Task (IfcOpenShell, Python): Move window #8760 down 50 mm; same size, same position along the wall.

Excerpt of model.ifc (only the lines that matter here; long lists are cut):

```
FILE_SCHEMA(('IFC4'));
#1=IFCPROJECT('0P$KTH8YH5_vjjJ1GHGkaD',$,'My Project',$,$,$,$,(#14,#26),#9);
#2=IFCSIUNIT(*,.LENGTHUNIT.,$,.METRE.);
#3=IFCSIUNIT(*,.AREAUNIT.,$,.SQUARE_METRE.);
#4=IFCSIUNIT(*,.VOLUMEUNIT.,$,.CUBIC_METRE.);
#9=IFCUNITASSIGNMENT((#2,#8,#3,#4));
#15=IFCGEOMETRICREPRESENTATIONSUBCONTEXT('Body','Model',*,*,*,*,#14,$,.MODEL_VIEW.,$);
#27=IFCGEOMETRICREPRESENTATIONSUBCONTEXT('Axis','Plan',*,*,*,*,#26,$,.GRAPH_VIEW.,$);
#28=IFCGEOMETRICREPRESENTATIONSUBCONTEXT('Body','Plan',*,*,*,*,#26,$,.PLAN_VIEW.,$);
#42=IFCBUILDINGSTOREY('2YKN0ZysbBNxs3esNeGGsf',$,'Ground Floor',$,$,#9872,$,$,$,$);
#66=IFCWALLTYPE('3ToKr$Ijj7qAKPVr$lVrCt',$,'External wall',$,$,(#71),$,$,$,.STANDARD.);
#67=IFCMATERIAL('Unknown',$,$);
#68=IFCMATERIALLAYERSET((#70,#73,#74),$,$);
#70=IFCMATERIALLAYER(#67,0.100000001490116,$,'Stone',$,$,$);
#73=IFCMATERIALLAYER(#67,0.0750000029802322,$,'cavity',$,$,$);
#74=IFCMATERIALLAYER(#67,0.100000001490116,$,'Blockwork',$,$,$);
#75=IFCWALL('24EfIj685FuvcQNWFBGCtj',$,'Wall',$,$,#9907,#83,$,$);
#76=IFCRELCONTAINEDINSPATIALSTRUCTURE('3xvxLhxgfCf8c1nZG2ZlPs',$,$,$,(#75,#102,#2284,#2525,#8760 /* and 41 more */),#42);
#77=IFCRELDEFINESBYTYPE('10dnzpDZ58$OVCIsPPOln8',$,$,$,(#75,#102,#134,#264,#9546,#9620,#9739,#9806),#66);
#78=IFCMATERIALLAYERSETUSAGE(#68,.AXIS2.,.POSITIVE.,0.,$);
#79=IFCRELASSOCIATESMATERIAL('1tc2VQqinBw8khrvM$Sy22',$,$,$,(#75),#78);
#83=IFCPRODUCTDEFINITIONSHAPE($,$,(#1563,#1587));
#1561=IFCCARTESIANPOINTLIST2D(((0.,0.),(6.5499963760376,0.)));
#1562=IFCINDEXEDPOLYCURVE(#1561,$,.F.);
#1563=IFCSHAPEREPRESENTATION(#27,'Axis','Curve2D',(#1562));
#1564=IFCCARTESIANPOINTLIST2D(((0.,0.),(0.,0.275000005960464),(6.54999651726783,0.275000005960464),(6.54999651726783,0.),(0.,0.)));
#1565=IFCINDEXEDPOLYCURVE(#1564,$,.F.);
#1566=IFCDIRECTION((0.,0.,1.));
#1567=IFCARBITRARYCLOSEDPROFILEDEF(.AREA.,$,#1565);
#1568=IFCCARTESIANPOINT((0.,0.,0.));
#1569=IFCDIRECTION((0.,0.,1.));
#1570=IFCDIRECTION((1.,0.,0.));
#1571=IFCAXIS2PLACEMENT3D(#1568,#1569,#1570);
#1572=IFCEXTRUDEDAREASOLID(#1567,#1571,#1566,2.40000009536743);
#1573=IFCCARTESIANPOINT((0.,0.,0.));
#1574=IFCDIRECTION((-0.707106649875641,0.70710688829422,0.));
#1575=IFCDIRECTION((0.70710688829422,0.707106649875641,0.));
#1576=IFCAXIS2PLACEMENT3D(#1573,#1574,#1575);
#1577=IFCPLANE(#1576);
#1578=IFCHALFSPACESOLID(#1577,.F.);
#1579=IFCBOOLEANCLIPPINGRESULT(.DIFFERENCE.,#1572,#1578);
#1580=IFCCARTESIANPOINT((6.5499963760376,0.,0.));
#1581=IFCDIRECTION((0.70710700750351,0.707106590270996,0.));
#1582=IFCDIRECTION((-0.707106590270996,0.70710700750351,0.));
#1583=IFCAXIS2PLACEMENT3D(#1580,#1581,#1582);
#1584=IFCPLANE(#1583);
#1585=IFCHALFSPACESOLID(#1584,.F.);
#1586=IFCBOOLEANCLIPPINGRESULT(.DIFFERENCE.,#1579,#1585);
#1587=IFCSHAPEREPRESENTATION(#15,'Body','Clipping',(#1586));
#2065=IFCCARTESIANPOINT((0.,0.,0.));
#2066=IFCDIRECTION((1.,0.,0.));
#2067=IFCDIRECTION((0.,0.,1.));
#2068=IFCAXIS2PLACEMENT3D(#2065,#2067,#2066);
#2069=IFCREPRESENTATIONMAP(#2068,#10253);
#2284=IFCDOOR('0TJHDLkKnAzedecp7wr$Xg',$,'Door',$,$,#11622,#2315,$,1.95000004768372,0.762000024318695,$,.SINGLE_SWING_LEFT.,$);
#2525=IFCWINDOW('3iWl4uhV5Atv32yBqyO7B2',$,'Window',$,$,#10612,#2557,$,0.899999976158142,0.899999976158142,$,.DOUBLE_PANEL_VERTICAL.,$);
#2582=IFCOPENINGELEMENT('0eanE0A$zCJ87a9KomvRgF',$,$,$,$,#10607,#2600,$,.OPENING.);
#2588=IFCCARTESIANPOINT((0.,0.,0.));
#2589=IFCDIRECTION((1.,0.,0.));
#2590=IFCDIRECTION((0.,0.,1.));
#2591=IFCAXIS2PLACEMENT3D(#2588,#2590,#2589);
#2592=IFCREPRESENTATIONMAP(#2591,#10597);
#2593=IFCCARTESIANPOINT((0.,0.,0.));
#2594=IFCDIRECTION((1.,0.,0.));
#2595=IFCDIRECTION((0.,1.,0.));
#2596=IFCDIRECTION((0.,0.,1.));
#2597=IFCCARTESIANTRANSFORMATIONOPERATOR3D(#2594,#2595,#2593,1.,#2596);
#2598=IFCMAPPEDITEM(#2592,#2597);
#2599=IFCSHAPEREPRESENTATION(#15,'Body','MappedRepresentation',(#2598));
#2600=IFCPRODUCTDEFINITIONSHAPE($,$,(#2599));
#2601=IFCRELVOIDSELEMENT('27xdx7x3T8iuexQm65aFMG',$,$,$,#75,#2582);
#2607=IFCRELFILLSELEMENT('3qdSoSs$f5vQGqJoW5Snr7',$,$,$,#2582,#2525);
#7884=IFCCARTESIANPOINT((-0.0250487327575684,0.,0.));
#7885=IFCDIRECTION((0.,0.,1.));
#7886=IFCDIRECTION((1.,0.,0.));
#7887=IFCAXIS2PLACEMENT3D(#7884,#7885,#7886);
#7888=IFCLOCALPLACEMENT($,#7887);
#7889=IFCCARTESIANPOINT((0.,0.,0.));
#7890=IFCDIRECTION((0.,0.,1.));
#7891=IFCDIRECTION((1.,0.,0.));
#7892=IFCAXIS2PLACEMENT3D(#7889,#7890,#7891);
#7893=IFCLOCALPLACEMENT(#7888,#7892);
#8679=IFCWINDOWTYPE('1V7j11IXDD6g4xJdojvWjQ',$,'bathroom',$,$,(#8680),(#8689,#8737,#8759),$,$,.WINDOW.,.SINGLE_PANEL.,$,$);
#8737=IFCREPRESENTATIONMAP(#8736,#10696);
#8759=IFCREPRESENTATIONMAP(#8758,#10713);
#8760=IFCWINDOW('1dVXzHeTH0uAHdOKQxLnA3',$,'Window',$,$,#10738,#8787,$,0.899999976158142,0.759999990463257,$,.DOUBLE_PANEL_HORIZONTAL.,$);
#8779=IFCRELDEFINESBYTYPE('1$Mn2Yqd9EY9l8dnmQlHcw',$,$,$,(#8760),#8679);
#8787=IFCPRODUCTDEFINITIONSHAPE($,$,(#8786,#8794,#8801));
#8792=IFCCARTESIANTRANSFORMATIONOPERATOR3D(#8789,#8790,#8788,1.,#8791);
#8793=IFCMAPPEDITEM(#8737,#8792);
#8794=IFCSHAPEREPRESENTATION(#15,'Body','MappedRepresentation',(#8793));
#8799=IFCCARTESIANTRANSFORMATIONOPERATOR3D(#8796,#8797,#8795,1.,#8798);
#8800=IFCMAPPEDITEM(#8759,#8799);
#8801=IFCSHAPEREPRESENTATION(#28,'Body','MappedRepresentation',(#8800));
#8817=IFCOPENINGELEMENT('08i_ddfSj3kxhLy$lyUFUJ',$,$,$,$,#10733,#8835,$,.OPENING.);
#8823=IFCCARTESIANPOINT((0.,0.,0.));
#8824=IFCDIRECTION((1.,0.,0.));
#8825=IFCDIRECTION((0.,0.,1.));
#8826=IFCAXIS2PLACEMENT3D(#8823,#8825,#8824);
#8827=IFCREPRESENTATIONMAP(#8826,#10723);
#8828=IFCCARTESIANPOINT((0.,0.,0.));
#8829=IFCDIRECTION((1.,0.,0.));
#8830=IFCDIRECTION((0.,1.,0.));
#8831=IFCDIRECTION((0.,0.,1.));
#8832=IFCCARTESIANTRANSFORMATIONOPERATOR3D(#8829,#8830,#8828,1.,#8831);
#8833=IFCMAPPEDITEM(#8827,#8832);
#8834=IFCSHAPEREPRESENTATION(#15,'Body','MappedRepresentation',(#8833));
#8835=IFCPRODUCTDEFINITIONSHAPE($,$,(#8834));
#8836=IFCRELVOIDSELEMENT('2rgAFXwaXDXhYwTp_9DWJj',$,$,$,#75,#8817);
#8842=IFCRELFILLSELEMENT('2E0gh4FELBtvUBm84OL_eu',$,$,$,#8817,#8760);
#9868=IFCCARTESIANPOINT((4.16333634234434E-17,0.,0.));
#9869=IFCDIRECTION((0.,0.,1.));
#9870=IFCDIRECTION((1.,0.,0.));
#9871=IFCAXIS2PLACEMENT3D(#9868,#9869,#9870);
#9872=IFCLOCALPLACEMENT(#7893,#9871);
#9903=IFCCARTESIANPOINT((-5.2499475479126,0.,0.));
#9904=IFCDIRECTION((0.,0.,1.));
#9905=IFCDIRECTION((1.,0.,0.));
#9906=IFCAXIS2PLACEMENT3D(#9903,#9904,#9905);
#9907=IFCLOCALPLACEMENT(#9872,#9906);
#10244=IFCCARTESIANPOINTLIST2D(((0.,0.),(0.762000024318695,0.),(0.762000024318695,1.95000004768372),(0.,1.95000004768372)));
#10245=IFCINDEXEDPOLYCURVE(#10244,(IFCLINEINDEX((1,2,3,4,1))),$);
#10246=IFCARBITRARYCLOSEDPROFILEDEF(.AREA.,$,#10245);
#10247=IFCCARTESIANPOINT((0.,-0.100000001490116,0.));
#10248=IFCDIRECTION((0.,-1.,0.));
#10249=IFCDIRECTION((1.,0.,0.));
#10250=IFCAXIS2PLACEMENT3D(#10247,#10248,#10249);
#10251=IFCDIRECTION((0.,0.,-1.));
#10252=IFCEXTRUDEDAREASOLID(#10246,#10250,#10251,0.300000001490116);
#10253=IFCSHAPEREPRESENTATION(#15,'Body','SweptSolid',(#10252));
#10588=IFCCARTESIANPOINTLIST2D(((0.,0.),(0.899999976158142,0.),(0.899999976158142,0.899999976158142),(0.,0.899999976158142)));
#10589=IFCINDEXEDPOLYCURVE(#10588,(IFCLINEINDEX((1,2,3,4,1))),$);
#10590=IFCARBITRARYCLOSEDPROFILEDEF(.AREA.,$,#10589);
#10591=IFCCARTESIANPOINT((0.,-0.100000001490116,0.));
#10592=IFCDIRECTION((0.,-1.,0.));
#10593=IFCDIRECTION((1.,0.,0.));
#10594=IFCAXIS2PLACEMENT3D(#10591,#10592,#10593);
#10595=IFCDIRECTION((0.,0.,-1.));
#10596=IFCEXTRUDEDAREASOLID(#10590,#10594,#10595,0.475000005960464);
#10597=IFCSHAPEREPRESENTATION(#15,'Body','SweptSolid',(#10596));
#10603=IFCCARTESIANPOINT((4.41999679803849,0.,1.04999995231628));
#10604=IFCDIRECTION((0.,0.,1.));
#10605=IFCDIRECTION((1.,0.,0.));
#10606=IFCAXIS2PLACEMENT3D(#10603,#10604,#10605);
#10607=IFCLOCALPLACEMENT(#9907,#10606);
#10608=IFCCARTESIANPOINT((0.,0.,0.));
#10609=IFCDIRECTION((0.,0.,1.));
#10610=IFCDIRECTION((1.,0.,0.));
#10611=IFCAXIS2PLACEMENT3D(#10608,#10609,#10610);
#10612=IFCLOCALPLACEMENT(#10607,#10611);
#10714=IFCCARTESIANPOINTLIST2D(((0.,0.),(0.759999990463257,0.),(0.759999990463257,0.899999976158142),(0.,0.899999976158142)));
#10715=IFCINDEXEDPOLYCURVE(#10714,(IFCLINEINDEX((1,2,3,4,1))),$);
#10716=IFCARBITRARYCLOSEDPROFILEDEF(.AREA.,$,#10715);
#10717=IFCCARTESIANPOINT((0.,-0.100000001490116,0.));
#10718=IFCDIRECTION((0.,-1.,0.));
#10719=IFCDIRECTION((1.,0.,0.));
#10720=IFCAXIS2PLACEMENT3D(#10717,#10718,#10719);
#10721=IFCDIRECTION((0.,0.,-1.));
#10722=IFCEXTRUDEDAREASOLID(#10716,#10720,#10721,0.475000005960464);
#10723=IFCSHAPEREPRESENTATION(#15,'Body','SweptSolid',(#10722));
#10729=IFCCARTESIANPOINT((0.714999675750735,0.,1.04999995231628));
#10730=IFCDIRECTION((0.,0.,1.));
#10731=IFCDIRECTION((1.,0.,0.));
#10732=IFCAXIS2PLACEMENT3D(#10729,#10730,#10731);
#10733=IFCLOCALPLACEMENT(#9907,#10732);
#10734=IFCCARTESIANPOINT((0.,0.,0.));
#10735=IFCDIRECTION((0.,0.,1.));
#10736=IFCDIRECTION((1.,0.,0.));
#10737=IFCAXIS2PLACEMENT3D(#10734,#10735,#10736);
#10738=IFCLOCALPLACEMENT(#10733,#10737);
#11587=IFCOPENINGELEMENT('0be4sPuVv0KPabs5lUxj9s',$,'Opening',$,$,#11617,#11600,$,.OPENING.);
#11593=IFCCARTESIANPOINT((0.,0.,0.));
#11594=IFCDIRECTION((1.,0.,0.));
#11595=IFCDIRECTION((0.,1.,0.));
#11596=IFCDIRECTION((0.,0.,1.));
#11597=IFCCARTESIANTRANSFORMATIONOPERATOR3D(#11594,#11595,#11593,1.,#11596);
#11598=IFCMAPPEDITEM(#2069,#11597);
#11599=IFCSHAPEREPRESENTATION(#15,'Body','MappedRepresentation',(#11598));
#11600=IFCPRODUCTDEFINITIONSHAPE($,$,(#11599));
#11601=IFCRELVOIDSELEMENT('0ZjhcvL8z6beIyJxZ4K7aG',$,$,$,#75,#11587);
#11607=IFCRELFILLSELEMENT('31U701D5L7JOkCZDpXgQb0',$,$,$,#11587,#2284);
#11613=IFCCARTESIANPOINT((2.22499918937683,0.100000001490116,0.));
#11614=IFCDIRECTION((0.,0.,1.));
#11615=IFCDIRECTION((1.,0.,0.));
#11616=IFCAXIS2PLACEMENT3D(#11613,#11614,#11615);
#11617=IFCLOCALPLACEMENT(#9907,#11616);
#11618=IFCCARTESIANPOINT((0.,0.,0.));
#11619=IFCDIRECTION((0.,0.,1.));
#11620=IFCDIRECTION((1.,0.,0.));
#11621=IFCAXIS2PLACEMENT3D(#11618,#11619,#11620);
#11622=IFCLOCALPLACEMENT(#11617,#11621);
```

```python
import numpy as np
import ifcopenshell
import ifcopenshell.api.geometry
import ifcopenshell.util.placement
import ifcopenshell.util.unit

model = ifcopenshell.open("model.ifc")
unit_scale = ifcopenshell.util.unit.calculate_unit_scale(model)

window = model.by_guid("1dVXzHeTH0uAHdOKQxLnA3")
opening = window.FillsVoids[0].RelatingOpeningElement
dz = -0.05 / unit_scale

shift = np.array([0.0, 0.0, dz])
# The window is placed relative to its opening, so it follows when the opening moves.
matrix = ifcopenshell.util.placement.get_local_placement(opening.ObjectPlacement)
matrix[:3, 3] += shift
ifcopenshell.api.geometry.edit_object_placement(
    model, product=opening, matrix=matrix, is_si=False, should_transform_children=True
)

print(f"moved by {dz * unit_scale:+.3f} m")

model.write("model_updated.ifc")
```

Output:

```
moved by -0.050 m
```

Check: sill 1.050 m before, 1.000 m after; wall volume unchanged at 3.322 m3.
